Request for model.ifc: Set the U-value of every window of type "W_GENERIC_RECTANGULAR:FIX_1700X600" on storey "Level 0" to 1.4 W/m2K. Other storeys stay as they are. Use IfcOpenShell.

First a look at what the model holds.

```python
import ifcopenshell
import ifcopenshell.util.element

model = ifcopenshell.open("model.ifc")
print(model.schema)
storey = next(s for s in model.by_type("IfcBuildingStorey") if s.Name == "Level 0")
windows = [e for e in ifcopenshell.util.element.get_decomposition(storey) if e.is_a("IfcWindow")]
seen = {}
for e in windows:
    element_type = ifcopenshell.util.element.get_type(e)
    key = (element_type.Name if element_type != e and element_type else None, ifcopenshell.util.element.get_pset(e, "Pset_WindowCommon", "ThermalTransmittance"))
    seen[key] = seen.get(key, 0) + 1
for (name, value), count in sorted(seen.items(), key=str):
    print(count, "x", name, "|", value)
```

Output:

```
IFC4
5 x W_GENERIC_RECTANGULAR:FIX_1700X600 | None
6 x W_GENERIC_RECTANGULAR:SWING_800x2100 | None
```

```python
import ifcopenshell
import ifcopenshell.api.pset
import ifcopenshell.util.element

model = ifcopenshell.open("model.ifc")

storey = next(s for s in model.by_type("IfcBuildingStorey") if s.Name == "Level 0")
windows = [e for e in ifcopenshell.util.element.get_decomposition(storey) if e.is_a("IfcWindow")]

count = 0
for e in windows:
    element_type = ifcopenshell.util.element.get_type(e)
    if element_type in (None, e) or element_type.Name != "W_GENERIC_RECTANGULAR:FIX_1700X600":
        continue
    # add_pset returns the element's existing set when there is one.
    pset = ifcopenshell.api.pset.add_pset(model, product=e, name="Pset_WindowCommon")
    ifcopenshell.api.pset.edit_pset(model, pset=pset, properties={"ThermalTransmittance": 1.4})
    count += 1

print(count, "windows updated")

model.write("model_rev.ifc")
```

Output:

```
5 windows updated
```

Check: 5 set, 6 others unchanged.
